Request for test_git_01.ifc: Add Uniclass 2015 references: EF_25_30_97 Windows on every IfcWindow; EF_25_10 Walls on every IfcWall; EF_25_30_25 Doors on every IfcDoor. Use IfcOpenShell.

First a look at what the model holds.

```python
import ifcopenshell

model = ifcopenshell.open("test_git_01.ifc")
print(model.schema)
print("classifications:", [c.Name for c in model.by_type("IfcClassification")])
for ifc_class in ("IfcDoor", "IfcRoof", "IfcStair", "IfcWall", "IfcWindow"):
    print(ifc_class, len(model.by_type(ifc_class)))
```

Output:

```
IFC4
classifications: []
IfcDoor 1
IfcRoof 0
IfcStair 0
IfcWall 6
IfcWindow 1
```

```python
import ifcopenshell
import ifcopenshell.api.classification

model = ifcopenshell.open("test_git_01.ifc")

system = ifcopenshell.api.classification.add_classification(model, classification="Uniclass 2015")

codes = {
    "IfcWindow": ("EF_25_30_97", "Windows"),
    "IfcWall": ("EF_25_10", "Walls"),
    "IfcDoor": ("EF_25_30_25", "Doors"),
}
for ifc_class, (code, name) in codes.items():
    products = model.by_type(ifc_class)
    ifcopenshell.api.classification.add_reference(
        model, products=products, classification=system, identification=code, name=name
    )
    print(code, len(products))

model.write("test_git_01_rev.ifc")
```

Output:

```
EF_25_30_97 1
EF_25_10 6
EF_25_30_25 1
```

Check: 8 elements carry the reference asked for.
